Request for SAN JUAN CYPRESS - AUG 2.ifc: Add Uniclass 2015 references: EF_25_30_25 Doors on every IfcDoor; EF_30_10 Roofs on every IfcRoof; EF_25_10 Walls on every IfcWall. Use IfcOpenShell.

First a look at what the model holds.

```python
import ifcopenshell

model = ifcopenshell.open("SAN JUAN CYPRESS - AUG 2.ifc")
print(model.schema)
print("classifications:", [c.Name for c in model.by_type("IfcClassification")])
for ifc_class in ("IfcDoor", "IfcRoof", "IfcStair", "IfcWall", "IfcWindow"):
    print(ifc_class, len(model.by_type(ifc_class)))
```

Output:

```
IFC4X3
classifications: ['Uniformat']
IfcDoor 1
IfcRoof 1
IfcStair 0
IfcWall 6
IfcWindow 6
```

```python
import ifcopenshell
import ifcopenshell.api.classification

model = ifcopenshell.open("SAN JUAN CYPRESS - AUG 2.ifc")

system = ifcopenshell.api.classification.add_classification(model, classification="Uniclass 2015")

codes = {
    "IfcDoor": ("EF_25_30_25", "Doors"),
    "IfcRoof": ("EF_30_10", "Roofs"),
    "IfcWall": ("EF_25_10", "Walls"),
}
for ifc_class, (code, name) in codes.items():
    products = model.by_type(ifc_class)
    ifcopenshell.api.classification.add_reference(
        model, products=products, classification=system, identification=code, name=name
    )
    print(code, len(products))

model.write("SAN JUAN CYPRESS - AUG 2_v2.ifc")
```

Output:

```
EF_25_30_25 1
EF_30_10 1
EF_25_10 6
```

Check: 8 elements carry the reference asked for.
